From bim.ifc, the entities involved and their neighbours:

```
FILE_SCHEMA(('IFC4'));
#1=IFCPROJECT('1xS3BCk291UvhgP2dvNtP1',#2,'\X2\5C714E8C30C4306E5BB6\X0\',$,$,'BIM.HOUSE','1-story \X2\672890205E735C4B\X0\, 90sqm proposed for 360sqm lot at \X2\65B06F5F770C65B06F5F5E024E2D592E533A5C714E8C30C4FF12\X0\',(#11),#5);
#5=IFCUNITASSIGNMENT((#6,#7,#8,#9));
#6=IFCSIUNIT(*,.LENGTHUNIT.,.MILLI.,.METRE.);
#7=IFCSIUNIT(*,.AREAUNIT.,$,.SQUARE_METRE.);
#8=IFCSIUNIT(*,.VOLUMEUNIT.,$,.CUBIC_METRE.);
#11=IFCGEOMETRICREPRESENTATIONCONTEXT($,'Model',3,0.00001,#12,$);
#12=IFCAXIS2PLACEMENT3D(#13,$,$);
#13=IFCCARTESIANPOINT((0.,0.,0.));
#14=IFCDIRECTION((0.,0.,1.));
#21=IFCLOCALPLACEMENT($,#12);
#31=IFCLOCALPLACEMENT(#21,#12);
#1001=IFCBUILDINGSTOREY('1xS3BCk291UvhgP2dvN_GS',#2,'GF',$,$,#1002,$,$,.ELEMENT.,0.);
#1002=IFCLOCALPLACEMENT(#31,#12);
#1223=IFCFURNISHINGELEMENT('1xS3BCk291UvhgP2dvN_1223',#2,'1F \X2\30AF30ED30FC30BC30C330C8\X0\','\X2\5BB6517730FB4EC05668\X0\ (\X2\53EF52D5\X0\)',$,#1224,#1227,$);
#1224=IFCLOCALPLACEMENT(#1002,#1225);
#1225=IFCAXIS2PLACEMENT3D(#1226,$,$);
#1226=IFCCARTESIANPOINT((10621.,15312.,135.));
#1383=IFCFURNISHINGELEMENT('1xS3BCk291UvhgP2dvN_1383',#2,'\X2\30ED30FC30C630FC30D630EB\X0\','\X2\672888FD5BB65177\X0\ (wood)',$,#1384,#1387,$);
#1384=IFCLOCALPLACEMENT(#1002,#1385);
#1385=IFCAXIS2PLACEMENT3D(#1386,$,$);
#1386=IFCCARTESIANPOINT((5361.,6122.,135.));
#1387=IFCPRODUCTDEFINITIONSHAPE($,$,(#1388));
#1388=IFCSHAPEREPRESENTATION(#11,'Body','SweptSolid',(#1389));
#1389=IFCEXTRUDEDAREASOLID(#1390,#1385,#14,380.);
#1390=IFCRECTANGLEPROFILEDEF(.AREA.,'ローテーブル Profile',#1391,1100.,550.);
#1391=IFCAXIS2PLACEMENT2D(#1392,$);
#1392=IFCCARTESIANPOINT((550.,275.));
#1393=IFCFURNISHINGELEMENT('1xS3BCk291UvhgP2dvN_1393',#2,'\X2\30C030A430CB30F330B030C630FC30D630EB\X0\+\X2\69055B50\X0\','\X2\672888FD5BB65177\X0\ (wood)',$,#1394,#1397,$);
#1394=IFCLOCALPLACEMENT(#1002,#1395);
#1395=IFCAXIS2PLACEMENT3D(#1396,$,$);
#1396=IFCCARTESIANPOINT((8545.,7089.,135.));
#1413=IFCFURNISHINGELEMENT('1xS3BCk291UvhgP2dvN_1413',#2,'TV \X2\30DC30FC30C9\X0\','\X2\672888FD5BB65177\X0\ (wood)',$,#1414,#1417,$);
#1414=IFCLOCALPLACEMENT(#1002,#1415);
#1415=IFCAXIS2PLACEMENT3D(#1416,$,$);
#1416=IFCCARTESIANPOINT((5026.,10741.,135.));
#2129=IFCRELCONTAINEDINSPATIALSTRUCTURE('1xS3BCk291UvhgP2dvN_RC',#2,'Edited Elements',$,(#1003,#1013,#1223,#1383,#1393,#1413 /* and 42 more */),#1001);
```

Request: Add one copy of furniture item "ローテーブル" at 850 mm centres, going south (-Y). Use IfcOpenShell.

```python
import numpy as np
import ifcopenshell
import ifcopenshell.api.geometry
import ifcopenshell.api.root
import ifcopenshell.util.element
import ifcopenshell.util.placement

model = ifcopenshell.open("bim.ifc")


def reuse_history(source, copy):
    """copy_class also copies each property set's owner history, people and application; keep the originals."""
    for rel in copy.IsDefinedBy:
        if rel.is_a("IfcRelDefinesByProperties") and (history := rel.RelatingPropertyDefinition.OwnerHistory):
            rel.RelatingPropertyDefinition.OwnerHistory = source.OwnerHistory
            ifcopenshell.util.element.remove_deep2(model, history)


source = model.by_guid("1xS3BCk291UvhgP2dvN_1383")
base = ifcopenshell.util.placement.get_local_placement(source.ObjectPlacement)
step = np.array([0.0, -1.0, 0.0]) * 850.0

for i in range(1, 2):
    copy = ifcopenshell.api.root.copy_class(model, product=source)
    copy.Representation = ifcopenshell.util.element.copy_deep(
        model, source.Representation, exclude=["IfcGeometricRepresentationContext", "IfcRepresentationMap"]
    )
    reuse_history(source, copy)
    matrix = base.copy()
    matrix[:3, 3] += i * step
    print("added at", matrix[:3, 3].round(3) + 0.0)
    ifcopenshell.api.geometry.edit_object_placement(model, product=copy, matrix=matrix, is_si=False)

model.write("bim_edited.ifc")
```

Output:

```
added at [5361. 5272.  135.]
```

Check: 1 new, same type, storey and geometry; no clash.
